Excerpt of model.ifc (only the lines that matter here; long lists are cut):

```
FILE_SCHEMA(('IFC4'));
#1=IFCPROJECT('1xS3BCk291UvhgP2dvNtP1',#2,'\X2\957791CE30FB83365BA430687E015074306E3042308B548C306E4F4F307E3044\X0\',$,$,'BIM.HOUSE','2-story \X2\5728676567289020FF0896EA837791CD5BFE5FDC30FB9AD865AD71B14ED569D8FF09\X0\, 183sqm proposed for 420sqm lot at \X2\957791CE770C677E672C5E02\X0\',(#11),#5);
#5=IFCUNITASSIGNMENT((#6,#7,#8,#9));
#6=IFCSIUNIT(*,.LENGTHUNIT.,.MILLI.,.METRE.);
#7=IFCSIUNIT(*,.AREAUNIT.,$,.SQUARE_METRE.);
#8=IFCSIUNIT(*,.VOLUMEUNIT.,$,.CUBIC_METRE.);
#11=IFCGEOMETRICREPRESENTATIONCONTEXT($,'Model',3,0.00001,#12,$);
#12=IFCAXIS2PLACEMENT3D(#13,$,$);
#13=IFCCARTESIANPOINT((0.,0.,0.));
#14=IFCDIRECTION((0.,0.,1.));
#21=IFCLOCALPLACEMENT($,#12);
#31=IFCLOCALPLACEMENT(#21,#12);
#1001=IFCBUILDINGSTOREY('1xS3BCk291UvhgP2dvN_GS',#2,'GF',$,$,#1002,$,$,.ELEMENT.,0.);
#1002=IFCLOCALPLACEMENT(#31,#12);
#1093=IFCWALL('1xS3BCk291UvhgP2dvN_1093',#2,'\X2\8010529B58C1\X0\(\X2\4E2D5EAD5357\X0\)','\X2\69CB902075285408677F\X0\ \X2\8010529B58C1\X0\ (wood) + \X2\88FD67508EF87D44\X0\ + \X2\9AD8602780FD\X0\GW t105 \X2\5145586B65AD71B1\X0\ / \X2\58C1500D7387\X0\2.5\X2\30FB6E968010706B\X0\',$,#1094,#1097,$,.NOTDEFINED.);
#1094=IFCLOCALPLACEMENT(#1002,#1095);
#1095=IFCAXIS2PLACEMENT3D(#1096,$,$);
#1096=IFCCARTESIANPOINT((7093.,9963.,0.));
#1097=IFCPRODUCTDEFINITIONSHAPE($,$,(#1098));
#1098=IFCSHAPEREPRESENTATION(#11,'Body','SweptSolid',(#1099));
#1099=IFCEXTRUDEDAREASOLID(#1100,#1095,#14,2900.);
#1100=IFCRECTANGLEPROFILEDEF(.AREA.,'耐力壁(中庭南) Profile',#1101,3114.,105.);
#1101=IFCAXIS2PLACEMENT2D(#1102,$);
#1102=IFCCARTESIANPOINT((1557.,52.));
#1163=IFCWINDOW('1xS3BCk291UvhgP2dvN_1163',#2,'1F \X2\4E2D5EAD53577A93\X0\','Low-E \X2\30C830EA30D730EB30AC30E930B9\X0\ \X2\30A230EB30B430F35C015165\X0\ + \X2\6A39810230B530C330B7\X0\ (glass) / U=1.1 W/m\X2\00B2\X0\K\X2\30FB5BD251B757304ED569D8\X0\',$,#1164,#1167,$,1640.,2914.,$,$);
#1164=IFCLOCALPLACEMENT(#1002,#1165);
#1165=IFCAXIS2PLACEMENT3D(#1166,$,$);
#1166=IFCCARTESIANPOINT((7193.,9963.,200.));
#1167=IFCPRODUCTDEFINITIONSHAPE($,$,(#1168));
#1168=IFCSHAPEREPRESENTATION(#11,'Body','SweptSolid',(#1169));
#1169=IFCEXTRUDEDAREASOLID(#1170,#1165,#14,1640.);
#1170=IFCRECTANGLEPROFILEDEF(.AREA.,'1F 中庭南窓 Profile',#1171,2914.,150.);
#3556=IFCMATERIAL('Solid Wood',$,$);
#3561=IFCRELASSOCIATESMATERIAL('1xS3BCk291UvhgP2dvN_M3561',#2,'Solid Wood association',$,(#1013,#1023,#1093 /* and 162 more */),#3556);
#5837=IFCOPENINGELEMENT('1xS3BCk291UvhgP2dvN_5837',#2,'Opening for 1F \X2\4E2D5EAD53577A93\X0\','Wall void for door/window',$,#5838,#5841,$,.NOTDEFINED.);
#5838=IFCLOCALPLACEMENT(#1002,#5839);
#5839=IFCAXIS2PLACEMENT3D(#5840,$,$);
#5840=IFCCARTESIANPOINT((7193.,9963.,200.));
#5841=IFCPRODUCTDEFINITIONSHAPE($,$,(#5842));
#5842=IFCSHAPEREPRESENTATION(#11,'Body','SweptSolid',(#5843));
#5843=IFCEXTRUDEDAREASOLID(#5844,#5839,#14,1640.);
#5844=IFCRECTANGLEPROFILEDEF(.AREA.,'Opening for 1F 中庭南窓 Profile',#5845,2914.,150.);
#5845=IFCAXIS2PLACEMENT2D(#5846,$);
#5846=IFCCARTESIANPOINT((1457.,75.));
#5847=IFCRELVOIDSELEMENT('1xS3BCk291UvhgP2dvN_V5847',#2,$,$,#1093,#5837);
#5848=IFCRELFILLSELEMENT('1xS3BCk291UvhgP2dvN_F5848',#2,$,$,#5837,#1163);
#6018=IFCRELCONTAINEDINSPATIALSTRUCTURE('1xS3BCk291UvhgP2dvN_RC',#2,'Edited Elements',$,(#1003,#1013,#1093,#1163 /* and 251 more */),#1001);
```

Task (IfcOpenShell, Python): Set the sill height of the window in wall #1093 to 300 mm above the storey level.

```python
import numpy as np
import ifcopenshell
import ifcopenshell.api.geometry
import ifcopenshell.geom
import ifcopenshell.util.element
import ifcopenshell.util.placement
import ifcopenshell.util.shape
import ifcopenshell.util.unit

model = ifcopenshell.open("model.ifc")
unit_scale = ifcopenshell.util.unit.calculate_unit_scale(model)

window = model.by_guid("1xS3BCk291UvhgP2dvN_1163")
opening = window.FillsVoids[0].RelatingOpeningElement
storey = ifcopenshell.util.element.get_container(window, ifc_class="IfcBuildingStorey")
level = ifcopenshell.util.placement.get_local_placement(storey.ObjectPlacement)[2, 3]

# The opening's origin need not be at the sill, so measure its lowest point.
shape = ifcopenshell.geom.create_shape(ifcopenshell.geom.settings(), opening)
bottom = ifcopenshell.util.shape.get_shape_bottom_elevation(shape, shape.geometry) / unit_scale
dz = level + 300.0 - bottom

shift = np.array([0.0, 0.0, dz])
# The window is not placed relative to its opening, so move both.
for product in (opening, window):
    matrix = ifcopenshell.util.placement.get_local_placement(product.ObjectPlacement)
    matrix[:3, 3] += shift
    ifcopenshell.api.geometry.edit_object_placement(model, product=product, matrix=matrix, is_si=False)

print(f"moved by {dz * unit_scale:+.3f} m")

model.write("model_updated.ifc")
```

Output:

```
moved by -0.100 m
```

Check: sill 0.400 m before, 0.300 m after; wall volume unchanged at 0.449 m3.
